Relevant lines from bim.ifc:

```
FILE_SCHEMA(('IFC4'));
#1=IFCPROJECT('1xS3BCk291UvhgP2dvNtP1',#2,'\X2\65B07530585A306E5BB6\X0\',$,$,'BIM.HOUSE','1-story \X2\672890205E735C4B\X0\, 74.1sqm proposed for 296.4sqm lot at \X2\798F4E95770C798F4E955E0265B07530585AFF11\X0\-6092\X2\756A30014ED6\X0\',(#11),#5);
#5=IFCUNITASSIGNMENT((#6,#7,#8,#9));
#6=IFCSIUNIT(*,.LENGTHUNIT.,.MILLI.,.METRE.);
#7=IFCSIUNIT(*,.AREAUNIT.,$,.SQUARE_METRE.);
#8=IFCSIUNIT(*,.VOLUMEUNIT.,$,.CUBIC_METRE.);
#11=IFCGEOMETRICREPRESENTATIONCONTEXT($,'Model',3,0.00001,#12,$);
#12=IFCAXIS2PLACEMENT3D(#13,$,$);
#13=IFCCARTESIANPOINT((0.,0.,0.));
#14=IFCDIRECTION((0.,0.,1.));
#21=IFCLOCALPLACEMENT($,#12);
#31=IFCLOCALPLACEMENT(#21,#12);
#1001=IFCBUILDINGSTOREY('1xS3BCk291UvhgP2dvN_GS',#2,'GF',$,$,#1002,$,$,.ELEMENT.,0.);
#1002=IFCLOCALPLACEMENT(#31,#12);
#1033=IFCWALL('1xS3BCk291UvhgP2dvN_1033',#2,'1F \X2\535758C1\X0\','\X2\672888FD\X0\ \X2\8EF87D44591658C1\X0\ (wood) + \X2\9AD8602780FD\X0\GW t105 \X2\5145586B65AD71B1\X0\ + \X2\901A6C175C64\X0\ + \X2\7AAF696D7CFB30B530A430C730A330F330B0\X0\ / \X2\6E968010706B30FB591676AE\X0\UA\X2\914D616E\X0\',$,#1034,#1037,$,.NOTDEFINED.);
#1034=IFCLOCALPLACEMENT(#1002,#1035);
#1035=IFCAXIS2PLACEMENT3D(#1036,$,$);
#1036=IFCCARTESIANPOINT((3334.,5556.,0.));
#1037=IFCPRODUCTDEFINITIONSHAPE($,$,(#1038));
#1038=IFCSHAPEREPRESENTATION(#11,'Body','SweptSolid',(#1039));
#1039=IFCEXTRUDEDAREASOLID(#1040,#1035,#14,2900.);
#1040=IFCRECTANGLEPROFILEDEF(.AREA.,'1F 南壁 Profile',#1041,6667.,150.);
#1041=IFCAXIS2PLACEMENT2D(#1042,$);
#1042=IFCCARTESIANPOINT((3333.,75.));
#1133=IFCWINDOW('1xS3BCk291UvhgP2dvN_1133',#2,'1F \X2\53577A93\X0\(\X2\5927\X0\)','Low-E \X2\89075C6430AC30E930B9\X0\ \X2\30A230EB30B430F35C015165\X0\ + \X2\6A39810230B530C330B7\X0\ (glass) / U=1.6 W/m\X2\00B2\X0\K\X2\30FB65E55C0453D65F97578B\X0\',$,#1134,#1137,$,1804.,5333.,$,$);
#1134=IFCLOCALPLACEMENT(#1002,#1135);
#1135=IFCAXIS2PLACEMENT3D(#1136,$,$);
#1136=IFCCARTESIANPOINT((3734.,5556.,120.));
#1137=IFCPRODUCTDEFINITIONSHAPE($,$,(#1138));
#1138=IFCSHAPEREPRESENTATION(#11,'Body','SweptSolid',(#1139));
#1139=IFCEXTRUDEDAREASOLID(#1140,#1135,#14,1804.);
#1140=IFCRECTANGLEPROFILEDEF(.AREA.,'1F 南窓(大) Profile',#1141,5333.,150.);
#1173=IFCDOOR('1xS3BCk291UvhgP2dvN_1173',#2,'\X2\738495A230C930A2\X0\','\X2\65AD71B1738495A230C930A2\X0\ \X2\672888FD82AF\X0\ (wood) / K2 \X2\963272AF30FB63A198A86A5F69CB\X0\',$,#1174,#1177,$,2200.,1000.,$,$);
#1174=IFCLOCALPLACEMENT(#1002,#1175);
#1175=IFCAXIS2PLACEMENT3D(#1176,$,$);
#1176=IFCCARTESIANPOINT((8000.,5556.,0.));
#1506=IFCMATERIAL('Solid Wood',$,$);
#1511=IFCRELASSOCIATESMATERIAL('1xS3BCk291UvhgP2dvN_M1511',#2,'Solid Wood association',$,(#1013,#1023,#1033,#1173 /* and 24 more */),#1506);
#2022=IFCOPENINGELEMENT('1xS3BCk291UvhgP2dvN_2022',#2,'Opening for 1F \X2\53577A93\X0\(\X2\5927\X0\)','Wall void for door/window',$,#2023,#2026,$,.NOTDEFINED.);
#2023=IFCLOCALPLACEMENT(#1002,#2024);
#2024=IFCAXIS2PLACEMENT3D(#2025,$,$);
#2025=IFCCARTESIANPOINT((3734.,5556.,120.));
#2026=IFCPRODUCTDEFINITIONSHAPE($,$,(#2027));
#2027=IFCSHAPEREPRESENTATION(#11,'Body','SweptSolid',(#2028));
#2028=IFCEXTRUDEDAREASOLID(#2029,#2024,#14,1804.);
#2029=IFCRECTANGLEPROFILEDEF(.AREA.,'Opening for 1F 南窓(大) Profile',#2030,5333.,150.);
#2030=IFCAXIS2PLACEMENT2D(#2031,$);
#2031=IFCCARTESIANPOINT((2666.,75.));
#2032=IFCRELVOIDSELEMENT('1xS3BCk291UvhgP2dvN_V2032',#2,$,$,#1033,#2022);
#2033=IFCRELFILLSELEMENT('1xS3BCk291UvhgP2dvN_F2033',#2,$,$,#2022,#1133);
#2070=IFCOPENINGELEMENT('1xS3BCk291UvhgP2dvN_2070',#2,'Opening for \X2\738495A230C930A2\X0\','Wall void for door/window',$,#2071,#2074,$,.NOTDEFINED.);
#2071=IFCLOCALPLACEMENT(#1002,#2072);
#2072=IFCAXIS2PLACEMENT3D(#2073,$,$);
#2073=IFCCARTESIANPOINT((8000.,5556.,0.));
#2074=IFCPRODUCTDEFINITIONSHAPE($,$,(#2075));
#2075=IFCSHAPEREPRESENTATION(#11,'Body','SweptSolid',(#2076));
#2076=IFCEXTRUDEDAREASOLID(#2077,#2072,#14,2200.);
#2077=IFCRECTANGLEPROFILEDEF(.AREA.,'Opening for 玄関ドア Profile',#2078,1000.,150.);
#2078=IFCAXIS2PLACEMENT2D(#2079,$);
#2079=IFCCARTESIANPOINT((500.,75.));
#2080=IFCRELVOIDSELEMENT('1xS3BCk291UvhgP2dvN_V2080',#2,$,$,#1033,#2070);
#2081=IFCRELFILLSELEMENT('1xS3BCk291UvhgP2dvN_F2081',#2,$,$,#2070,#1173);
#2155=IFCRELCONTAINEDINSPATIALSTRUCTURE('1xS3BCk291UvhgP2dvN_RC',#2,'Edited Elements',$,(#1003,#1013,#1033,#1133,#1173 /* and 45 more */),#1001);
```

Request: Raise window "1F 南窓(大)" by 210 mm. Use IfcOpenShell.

```python
import numpy as np
import ifcopenshell
import ifcopenshell.api.geometry
import ifcopenshell.util.placement
import ifcopenshell.util.unit

model = ifcopenshell.open("bim.ifc")
unit_scale = ifcopenshell.util.unit.calculate_unit_scale(model)

window = model.by_id(1133)
opening = window.FillsVoids[0].RelatingOpeningElement
dz = 0.21 / unit_scale

shift = np.array([0.0, 0.0, dz])
# The window is not placed relative to its opening, so move both.
for product in (opening, window):
    matrix = ifcopenshell.util.placement.get_local_placement(product.ObjectPlacement)
    matrix[:3, 3] += shift
    ifcopenshell.api.geometry.edit_object_placement(model, product=product, matrix=matrix, is_si=False)

print(f"moved by {dz * unit_scale:+.3f} m")

model.write("bim_v2.ifc")
```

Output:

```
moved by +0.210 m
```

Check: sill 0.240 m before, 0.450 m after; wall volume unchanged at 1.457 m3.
